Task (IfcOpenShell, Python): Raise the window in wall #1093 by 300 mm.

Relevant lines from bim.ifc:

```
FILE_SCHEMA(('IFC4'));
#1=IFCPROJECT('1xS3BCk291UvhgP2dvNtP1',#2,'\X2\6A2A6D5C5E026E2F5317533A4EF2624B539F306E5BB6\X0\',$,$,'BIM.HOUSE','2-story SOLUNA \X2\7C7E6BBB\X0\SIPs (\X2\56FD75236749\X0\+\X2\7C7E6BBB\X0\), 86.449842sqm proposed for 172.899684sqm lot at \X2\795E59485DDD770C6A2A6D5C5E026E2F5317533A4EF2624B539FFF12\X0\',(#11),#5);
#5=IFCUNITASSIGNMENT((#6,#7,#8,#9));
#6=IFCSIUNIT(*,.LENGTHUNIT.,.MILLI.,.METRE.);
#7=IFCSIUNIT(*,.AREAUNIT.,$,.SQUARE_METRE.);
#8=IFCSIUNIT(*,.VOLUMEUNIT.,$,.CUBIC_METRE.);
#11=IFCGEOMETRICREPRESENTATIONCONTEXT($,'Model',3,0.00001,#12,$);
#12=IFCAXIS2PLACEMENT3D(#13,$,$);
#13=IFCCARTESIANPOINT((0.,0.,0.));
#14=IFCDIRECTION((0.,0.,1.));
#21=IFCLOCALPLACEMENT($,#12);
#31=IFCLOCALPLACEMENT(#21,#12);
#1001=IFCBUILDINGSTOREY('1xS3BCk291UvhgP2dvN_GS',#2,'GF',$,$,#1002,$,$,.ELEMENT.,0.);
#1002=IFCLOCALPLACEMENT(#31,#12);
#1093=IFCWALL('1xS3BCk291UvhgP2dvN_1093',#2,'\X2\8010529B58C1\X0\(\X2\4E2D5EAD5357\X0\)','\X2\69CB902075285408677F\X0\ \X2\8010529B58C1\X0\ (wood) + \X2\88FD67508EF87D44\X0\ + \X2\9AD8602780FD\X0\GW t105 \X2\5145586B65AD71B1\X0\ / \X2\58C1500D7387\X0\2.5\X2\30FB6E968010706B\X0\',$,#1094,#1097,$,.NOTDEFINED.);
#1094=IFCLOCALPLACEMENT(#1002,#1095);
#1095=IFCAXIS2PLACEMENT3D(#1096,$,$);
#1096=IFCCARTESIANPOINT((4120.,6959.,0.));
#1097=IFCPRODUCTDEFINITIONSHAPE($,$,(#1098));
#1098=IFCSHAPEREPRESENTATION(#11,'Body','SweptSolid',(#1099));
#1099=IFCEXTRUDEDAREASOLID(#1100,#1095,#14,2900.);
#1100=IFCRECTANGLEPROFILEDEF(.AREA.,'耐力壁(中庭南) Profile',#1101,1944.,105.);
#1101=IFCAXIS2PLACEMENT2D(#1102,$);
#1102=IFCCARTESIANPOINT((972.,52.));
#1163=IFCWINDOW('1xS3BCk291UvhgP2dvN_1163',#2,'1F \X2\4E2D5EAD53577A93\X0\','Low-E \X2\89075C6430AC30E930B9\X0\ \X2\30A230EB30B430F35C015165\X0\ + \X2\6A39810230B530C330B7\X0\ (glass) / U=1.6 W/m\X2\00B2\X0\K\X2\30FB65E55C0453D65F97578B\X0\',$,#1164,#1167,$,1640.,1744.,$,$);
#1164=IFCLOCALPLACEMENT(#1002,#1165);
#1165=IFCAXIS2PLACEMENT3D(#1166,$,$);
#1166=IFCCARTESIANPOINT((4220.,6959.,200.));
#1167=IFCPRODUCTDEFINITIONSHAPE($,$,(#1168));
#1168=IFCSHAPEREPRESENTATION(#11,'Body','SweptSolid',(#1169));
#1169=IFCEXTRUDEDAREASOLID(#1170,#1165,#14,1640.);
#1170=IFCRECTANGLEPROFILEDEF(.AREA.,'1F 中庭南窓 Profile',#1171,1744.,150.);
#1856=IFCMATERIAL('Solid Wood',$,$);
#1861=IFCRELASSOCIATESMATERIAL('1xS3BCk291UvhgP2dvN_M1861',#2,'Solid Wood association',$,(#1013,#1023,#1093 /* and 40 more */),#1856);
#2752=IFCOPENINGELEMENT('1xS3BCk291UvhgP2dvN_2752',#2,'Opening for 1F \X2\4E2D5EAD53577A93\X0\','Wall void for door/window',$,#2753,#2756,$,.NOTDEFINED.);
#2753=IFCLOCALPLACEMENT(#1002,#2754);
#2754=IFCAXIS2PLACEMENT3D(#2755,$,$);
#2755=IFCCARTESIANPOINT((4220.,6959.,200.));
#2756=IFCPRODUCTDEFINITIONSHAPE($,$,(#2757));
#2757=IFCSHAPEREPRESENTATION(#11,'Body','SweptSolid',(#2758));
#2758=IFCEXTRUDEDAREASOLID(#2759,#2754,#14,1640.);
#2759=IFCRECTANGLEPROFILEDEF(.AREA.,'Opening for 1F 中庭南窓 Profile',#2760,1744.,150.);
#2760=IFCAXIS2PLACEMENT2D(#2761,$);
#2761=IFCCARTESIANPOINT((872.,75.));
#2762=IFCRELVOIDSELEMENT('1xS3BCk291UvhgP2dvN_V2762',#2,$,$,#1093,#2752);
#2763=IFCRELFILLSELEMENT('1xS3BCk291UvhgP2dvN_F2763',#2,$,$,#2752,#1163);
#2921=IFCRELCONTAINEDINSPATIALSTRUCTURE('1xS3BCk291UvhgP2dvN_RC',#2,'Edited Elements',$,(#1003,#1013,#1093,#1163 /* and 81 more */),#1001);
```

```python
import numpy as np
import ifcopenshell
import ifcopenshell.api.geometry
import ifcopenshell.util.placement
import ifcopenshell.util.unit

model = ifcopenshell.open("bim.ifc")
unit_scale = ifcopenshell.util.unit.calculate_unit_scale(model)

window = model.by_guid("1xS3BCk291UvhgP2dvN_1163")
opening = window.FillsVoids[0].RelatingOpeningElement
dz = 300.0

shift = np.array([0.0, 0.0, dz])
# The window is not placed relative to its opening, so move both.
for product in (opening, window):
    matrix = ifcopenshell.util.placement.get_local_placement(product.ObjectPlacement)
    matrix[:3, 3] += shift
    ifcopenshell.api.geometry.edit_object_placement(model, product=product, matrix=matrix, is_si=False)

print(f"moved by {dz * unit_scale:+.3f} m")

model.write("bim-out.ifc")
```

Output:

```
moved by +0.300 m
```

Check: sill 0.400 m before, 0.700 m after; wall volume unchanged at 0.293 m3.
